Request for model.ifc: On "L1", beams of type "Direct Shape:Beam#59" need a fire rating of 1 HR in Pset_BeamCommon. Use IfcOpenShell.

First a look at what the model holds.

```python
import ifcopenshell
import ifcopenshell.util.element

model = ifcopenshell.open("model.ifc")
print(model.schema)
storey = next(s for s in model.by_type("IfcBuildingStorey") if s.Name == "L1")
beams = [e for e in ifcopenshell.util.element.get_decomposition(storey) if e.is_a("IfcBeam")]
seen = {}
for e in beams:
    element_type = ifcopenshell.util.element.get_type(e)
    key = (element_type.Name if element_type != e and element_type else None, ifcopenshell.util.element.get_pset(e, "Pset_BeamCommon", "FireRating"))
    seen[key] = seen.get(key, 0) + 1
for (name, value), count in sorted(seen.items(), key=str):
    print(count, "x", name, "|", value)
```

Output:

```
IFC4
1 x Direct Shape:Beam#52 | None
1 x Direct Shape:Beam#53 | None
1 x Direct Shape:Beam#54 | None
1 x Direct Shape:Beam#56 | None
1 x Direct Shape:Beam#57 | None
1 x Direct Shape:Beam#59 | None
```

```python
import ifcopenshell
import ifcopenshell.api.pset
import ifcopenshell.util.element

model = ifcopenshell.open("model.ifc")

storey = next(s for s in model.by_type("IfcBuildingStorey") if s.Name == "L1")
beams = [e for e in ifcopenshell.util.element.get_decomposition(storey) if e.is_a("IfcBeam")]

count = 0
for e in beams:
    element_type = ifcopenshell.util.element.get_type(e)
    if element_type in (None, e) or element_type.Name != "Direct Shape:Beam#59":
        continue
    # add_pset returns the element's existing set when there is one.
    pset = ifcopenshell.api.pset.add_pset(model, product=e, name="Pset_BeamCommon")
    ifcopenshell.api.pset.edit_pset(model, pset=pset, properties={"FireRating": "1 HR"})
    count += 1

print(count, "beams updated")

model.write("model_v2.ifc")
```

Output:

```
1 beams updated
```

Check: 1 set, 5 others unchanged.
